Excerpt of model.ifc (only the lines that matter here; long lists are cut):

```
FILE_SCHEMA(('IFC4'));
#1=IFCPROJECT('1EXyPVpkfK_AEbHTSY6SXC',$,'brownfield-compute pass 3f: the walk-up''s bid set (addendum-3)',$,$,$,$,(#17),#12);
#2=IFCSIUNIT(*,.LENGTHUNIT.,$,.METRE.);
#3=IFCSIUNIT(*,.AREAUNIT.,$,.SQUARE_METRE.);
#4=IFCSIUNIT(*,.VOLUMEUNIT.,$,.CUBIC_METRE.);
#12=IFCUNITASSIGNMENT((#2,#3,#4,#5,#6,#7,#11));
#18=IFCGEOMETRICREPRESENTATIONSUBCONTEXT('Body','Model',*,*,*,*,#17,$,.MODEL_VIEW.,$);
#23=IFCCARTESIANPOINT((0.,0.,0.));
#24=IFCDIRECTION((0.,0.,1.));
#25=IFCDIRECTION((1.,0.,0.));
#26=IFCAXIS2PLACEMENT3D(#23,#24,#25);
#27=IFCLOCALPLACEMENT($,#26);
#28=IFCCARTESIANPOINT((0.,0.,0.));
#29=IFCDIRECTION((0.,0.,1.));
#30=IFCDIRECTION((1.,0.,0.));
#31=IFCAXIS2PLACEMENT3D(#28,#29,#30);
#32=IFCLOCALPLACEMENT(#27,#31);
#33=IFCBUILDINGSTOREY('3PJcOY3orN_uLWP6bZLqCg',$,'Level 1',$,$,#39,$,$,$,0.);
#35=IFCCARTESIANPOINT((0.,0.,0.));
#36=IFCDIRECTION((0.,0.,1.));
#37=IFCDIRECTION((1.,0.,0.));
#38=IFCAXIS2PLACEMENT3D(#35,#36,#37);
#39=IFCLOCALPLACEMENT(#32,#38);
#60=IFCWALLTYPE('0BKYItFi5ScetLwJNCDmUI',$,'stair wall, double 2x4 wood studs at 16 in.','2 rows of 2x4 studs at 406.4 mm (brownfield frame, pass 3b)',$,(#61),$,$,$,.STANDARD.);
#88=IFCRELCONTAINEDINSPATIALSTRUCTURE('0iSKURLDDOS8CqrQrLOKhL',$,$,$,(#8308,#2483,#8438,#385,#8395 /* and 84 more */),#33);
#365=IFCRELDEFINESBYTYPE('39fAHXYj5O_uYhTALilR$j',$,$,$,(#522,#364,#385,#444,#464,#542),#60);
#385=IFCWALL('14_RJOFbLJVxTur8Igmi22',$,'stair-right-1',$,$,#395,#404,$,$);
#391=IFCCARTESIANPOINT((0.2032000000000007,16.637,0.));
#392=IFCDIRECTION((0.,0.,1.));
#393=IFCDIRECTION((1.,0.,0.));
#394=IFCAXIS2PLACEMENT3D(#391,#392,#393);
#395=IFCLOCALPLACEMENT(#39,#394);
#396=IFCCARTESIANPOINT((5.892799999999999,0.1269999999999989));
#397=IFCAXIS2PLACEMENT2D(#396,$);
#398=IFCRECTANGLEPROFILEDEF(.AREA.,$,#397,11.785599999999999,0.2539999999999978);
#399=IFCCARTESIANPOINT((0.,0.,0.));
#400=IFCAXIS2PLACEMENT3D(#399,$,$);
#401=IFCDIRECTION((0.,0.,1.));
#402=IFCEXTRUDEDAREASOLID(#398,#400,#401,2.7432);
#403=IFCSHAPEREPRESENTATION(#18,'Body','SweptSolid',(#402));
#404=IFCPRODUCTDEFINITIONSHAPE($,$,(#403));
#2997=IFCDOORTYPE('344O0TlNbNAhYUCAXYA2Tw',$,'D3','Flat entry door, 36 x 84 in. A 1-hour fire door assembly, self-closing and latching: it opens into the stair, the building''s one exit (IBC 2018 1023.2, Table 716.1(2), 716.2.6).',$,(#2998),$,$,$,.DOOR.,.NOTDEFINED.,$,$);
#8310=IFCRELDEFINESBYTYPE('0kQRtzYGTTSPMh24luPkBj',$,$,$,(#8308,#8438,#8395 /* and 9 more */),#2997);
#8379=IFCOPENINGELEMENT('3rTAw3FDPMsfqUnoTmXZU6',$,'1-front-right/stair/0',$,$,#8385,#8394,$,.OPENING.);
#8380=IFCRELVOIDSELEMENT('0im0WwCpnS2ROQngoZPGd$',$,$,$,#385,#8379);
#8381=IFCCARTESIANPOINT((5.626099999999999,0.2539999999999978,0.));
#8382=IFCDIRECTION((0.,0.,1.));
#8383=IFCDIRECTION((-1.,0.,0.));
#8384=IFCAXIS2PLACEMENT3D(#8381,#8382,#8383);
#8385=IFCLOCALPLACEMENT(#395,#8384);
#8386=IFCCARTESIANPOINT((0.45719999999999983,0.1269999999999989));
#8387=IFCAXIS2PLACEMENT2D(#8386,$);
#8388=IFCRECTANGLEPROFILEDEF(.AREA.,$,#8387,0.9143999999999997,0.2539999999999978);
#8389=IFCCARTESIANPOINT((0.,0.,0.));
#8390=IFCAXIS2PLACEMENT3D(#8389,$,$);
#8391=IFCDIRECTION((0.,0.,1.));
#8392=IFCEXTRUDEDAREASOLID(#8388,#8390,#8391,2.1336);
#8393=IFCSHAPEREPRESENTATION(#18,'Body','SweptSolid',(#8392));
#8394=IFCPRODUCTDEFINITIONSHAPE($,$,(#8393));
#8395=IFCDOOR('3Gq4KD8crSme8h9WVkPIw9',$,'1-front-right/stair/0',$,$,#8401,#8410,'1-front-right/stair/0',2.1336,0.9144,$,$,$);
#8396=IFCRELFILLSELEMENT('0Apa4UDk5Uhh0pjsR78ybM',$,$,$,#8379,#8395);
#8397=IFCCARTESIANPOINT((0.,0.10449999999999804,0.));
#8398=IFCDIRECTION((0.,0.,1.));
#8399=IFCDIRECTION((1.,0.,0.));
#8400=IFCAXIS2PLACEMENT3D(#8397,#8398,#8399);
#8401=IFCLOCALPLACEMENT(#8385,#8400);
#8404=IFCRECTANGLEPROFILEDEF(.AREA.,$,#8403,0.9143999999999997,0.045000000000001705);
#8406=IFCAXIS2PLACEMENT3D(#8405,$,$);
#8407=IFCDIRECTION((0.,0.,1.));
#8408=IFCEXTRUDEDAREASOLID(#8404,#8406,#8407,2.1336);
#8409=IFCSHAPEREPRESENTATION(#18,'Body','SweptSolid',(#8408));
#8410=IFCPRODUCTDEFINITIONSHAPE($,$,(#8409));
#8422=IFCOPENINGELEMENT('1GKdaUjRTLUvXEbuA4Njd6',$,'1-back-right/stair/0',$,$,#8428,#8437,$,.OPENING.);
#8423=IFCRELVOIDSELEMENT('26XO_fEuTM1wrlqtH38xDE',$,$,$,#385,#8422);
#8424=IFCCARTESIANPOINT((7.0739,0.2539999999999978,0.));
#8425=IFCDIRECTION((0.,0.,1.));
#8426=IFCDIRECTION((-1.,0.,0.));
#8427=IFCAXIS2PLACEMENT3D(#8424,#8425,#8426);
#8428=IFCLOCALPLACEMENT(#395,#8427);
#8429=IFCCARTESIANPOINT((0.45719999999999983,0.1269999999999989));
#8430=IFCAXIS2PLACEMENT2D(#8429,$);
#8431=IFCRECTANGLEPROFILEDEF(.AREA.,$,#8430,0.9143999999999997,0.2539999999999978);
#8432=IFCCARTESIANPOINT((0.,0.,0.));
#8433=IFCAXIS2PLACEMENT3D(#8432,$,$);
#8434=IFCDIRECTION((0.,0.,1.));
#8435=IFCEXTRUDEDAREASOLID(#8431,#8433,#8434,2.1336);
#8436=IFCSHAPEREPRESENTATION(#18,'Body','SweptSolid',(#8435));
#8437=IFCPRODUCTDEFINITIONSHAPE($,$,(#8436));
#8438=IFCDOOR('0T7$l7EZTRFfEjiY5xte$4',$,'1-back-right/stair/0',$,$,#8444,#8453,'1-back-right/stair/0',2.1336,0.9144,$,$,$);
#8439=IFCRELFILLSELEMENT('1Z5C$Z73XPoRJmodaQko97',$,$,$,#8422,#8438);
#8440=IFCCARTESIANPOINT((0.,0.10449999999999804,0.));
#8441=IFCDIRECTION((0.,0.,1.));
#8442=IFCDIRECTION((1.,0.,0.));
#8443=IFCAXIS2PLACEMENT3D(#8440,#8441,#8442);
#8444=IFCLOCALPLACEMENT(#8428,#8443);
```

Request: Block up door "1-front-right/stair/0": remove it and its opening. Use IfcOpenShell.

```python
import ifcopenshell
import ifcopenshell.api.feature
import ifcopenshell.api.root
import ifcopenshell.geom
import ifcopenshell.util.shape

model = ifcopenshell.open("model.ifc")
settings = ifcopenshell.geom.settings()


def volume(element):
    """Net volume in cubic metres, openings subtracted."""
    shape = ifcopenshell.geom.create_shape(settings, element)
    return ifcopenshell.util.shape.get_volume(shape.geometry)


door = model.by_guid("3Gq4KD8crSme8h9WVkPIw9")
opening = door.FillsVoids[0].RelatingOpeningElement
wall = opening.VoidsElements[0].RelatingBuildingElement
before = volume(wall)

ifcopenshell.api.root.remove_product(model, product=door)
ifcopenshell.api.feature.remove_feature(model, feature=opening)

after = volume(wall)

print(f"wall volume {before:.3f} -> {after:.3f} m3")

model.write("model-out.ifc")
```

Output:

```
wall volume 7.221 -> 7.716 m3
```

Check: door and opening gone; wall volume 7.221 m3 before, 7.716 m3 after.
